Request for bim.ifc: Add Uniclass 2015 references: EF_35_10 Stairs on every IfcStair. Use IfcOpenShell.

First a look at what the model holds.

```python
import ifcopenshell

model = ifcopenshell.open("bim.ifc")
print(model.schema)
print("classifications:", [c.Name for c in model.by_type("IfcClassification")])
for ifc_class in ("IfcDoor", "IfcRoof", "IfcStair", "IfcWall", "IfcWindow"):
    print(ifc_class, len(model.by_type(ifc_class)))
```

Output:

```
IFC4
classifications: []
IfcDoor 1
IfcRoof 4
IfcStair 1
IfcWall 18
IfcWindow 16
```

```python
import ifcopenshell
import ifcopenshell.api.classification

model = ifcopenshell.open("bim.ifc")

system = ifcopenshell.api.classification.add_classification(model, classification="Uniclass 2015")

codes = {
    "IfcStair": ("EF_35_10", "Stairs"),
}
for ifc_class, (code, name) in codes.items():
    products = model.by_type(ifc_class)
    ifcopenshell.api.classification.add_reference(
        model, products=products, classification=system, identification=code, name=name
    )
    print(code, len(products))

model.write("bim_updated.ifc")
```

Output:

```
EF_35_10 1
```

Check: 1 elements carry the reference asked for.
